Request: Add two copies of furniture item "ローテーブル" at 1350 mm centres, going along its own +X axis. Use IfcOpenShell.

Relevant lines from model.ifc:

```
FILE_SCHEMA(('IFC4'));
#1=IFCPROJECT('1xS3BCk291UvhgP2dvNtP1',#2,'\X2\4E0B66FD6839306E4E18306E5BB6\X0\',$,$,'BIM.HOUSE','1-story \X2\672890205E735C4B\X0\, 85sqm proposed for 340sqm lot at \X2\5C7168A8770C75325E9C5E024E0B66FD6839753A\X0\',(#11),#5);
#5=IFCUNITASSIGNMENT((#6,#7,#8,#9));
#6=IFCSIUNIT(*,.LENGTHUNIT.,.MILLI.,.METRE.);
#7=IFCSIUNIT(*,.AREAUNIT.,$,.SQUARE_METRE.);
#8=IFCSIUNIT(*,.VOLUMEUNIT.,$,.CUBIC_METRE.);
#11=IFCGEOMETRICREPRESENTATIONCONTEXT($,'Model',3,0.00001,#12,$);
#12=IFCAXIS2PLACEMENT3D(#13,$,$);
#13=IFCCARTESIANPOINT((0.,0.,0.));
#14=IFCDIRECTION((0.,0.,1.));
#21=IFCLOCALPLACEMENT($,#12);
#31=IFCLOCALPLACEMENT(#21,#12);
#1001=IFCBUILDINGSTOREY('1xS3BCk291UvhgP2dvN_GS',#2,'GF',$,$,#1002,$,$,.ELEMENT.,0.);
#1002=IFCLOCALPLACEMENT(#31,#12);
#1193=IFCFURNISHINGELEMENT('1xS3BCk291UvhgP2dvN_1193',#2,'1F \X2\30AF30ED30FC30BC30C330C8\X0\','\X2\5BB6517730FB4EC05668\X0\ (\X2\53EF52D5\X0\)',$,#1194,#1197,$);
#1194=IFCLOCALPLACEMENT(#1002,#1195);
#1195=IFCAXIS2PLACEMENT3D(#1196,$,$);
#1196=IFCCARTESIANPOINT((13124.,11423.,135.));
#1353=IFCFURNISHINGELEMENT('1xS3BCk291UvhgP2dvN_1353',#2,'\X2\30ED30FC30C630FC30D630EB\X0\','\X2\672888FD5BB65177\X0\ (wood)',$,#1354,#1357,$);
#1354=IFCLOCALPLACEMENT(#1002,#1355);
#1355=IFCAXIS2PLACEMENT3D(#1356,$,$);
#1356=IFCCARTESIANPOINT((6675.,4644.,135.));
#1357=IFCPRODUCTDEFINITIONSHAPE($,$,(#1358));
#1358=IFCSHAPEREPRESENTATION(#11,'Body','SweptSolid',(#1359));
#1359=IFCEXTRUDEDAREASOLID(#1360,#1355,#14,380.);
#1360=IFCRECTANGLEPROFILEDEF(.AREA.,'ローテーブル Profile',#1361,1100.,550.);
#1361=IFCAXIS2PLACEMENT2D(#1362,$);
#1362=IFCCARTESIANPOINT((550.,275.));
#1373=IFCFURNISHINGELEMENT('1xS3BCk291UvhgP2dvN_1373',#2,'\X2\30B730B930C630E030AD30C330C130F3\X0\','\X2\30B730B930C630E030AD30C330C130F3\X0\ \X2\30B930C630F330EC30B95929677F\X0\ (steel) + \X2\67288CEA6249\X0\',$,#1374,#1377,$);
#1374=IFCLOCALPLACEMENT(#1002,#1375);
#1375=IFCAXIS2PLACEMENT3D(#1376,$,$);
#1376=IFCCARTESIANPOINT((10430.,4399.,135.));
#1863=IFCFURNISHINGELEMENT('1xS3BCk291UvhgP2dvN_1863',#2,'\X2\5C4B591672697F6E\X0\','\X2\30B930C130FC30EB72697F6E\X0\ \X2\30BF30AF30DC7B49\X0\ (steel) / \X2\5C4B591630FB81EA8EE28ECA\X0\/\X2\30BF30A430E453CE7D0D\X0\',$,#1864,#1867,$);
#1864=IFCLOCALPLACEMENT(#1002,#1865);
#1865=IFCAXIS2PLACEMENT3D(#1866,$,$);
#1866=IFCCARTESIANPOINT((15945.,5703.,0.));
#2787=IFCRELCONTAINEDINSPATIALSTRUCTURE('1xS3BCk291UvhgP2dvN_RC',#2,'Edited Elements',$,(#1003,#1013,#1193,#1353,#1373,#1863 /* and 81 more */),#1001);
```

```python
import ifcopenshell
import ifcopenshell.api.geometry
import ifcopenshell.api.root
import ifcopenshell.util.element
import ifcopenshell.util.placement

model = ifcopenshell.open("model.ifc")


def reuse_history(source, copy):
    """copy_class also copies each property set's owner history, people and application; keep the originals."""
    for rel in copy.IsDefinedBy:
        if rel.is_a("IfcRelDefinesByProperties") and (history := rel.RelatingPropertyDefinition.OwnerHistory):
            rel.RelatingPropertyDefinition.OwnerHistory = source.OwnerHistory
            ifcopenshell.util.element.remove_deep2(model, history)


source = model.by_guid("1xS3BCk291UvhgP2dvN_1353")
base = ifcopenshell.util.placement.get_local_placement(source.ObjectPlacement)
step = base[:3, 0] * 1350.0

for i in range(1, 3):
    copy = ifcopenshell.api.root.copy_class(model, product=source)
    copy.Representation = ifcopenshell.util.element.copy_deep(
        model, source.Representation, exclude=["IfcGeometricRepresentationContext", "IfcRepresentationMap"]
    )
    reuse_history(source, copy)
    matrix = base.copy()
    matrix[:3, 3] += i * step
    print("added at", matrix[:3, 3].round(3) + 0.0)
    ifcopenshell.api.geometry.edit_object_placement(model, product=copy, matrix=matrix, is_si=False)

model.write("model_edited.ifc")
```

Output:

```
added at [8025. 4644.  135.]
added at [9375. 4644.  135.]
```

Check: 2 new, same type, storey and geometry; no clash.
